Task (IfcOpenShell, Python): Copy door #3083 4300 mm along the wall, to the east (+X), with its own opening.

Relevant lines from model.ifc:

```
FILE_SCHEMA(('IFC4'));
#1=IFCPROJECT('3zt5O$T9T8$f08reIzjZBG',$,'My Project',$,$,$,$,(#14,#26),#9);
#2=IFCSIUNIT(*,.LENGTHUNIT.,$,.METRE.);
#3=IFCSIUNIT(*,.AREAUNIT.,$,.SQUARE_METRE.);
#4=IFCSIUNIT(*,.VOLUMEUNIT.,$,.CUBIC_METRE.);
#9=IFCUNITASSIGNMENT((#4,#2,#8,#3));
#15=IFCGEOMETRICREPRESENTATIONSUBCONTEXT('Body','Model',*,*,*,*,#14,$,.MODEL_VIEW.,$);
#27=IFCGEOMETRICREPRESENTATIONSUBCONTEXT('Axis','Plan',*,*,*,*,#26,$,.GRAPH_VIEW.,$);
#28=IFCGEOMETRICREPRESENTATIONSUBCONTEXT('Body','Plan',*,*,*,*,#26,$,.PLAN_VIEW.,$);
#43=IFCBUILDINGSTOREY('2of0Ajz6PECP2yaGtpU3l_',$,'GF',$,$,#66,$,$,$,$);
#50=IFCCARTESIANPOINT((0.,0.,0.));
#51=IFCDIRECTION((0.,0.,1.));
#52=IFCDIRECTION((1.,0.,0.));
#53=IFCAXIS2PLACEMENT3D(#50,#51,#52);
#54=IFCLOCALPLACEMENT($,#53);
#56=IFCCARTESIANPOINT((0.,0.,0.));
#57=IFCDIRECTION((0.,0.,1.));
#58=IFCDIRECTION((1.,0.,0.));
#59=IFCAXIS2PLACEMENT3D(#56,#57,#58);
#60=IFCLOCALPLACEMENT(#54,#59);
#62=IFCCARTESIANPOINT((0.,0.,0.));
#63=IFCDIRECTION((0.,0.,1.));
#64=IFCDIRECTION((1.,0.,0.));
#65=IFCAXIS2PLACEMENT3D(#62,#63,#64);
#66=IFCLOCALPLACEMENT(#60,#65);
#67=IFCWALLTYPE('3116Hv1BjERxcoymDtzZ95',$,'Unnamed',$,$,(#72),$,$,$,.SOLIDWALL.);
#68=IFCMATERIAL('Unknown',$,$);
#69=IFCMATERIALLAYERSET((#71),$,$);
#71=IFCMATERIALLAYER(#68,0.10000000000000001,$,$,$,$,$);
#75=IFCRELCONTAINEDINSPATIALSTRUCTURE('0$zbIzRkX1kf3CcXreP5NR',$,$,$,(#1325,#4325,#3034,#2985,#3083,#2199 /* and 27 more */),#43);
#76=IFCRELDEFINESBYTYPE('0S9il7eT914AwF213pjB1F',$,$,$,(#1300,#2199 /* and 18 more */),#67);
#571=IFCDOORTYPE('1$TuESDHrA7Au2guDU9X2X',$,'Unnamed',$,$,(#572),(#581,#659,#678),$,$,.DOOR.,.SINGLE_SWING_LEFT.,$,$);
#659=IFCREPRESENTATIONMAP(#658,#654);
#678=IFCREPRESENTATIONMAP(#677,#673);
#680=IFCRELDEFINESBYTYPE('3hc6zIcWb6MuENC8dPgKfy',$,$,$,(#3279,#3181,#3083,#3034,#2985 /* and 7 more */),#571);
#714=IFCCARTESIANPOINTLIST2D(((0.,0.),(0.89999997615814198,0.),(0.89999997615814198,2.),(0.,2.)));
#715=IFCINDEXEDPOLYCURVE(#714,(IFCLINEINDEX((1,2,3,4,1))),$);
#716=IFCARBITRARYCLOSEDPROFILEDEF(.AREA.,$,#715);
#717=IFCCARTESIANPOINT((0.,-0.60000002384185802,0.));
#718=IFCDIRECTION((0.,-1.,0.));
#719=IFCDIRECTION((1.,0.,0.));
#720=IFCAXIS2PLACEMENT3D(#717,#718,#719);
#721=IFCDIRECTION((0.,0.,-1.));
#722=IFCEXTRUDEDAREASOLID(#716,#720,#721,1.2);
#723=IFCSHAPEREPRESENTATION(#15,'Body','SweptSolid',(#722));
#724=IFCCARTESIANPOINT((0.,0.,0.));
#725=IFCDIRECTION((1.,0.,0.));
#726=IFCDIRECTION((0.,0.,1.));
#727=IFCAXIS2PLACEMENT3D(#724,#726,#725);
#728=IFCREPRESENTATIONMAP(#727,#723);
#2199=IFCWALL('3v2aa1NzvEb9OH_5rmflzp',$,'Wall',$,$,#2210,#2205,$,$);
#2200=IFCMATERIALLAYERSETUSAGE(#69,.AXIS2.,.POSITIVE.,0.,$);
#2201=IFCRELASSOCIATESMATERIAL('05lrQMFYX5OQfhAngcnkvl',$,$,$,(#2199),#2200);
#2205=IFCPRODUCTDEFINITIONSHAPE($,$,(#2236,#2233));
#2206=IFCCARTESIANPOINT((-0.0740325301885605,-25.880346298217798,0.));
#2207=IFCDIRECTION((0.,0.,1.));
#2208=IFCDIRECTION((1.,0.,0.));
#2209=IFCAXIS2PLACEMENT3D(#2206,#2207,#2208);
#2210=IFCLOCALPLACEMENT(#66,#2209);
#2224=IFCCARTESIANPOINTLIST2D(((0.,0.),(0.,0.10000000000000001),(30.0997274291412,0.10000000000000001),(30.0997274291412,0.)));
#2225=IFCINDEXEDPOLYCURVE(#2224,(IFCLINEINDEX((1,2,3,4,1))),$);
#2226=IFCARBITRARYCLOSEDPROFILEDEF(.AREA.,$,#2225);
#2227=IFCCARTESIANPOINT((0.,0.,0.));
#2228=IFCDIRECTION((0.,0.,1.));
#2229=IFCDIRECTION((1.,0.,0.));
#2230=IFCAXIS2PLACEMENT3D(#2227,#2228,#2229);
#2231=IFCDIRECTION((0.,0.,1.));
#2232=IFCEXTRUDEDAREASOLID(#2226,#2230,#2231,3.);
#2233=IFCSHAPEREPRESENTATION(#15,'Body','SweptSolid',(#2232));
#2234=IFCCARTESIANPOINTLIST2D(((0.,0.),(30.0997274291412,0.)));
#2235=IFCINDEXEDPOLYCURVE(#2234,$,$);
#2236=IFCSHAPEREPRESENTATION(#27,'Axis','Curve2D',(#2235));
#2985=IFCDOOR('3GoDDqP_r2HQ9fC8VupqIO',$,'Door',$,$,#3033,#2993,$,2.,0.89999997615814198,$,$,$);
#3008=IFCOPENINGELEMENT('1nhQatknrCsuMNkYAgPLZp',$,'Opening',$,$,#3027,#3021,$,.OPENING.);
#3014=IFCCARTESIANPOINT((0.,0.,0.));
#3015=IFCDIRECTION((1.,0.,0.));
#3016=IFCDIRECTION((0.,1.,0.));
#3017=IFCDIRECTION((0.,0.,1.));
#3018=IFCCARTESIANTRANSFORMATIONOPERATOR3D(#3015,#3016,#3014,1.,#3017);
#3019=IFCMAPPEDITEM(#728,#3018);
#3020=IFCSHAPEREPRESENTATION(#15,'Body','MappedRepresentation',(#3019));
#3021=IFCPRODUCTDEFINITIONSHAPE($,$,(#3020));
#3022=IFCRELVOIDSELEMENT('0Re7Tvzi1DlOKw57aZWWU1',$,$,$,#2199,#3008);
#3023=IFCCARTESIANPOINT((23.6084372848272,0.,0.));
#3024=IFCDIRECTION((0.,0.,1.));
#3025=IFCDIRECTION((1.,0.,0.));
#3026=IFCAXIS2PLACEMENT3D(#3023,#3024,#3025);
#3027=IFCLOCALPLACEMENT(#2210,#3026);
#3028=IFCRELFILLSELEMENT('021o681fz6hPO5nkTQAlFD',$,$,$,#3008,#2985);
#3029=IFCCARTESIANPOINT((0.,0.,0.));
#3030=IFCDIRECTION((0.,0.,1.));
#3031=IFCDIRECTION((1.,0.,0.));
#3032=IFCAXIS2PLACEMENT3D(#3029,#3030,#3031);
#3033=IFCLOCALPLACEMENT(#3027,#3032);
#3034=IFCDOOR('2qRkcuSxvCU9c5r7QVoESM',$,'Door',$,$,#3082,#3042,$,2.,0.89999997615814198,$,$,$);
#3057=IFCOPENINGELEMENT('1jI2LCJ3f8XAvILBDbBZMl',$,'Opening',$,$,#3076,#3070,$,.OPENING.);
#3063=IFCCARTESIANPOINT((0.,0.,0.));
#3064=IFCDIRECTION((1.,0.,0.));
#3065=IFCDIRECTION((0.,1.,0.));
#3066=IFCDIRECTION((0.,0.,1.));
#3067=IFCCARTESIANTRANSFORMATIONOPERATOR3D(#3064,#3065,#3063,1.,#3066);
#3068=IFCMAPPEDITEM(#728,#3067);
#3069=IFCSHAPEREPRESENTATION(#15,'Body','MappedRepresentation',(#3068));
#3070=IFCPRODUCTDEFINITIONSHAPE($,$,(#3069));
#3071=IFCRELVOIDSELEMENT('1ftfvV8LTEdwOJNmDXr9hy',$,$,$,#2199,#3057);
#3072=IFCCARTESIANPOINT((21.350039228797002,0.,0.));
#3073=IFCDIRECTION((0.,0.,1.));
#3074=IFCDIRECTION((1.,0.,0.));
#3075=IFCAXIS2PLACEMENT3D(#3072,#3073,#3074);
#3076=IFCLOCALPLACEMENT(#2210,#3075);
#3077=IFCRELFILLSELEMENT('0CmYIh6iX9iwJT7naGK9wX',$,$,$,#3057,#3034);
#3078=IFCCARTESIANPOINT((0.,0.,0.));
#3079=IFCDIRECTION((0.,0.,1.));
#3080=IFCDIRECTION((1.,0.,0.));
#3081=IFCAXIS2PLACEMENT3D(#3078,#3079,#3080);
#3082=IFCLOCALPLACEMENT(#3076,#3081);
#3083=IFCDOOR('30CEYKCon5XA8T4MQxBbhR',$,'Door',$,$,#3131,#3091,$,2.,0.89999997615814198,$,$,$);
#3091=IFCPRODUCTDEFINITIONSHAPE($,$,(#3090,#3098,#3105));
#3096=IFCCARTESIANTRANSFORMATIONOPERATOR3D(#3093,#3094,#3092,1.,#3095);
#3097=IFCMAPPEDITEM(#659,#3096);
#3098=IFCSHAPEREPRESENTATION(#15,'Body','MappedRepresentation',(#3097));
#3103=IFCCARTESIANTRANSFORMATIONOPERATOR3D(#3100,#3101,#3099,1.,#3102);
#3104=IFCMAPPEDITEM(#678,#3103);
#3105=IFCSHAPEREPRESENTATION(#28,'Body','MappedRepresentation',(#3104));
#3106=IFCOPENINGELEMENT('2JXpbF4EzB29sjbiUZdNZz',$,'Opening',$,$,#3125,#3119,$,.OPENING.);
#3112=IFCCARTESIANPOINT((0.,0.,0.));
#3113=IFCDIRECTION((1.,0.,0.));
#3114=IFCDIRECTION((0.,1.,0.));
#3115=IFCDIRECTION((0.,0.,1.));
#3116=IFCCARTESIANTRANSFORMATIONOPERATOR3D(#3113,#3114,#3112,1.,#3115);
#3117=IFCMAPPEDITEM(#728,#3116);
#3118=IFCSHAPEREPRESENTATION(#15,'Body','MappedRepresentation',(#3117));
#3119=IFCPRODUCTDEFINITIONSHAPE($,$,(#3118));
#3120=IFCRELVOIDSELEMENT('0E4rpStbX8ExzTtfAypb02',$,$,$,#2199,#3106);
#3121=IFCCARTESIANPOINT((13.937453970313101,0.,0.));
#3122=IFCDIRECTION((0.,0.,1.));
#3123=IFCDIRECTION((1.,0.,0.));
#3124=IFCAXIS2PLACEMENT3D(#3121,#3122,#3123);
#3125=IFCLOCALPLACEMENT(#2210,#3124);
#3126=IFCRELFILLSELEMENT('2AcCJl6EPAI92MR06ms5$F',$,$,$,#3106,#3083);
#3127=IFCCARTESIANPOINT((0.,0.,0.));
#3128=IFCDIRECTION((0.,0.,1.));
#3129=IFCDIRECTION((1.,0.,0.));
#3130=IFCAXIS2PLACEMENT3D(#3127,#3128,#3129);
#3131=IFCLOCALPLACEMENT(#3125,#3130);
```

```python
import ifcopenshell
import ifcopenshell.api.feature
import ifcopenshell.api.geometry
import ifcopenshell.api.root
import ifcopenshell.geom
import ifcopenshell.util.element
import ifcopenshell.util.placement
import ifcopenshell.util.shape
import ifcopenshell.util.unit

model = ifcopenshell.open("model.ifc")
unit_scale = ifcopenshell.util.unit.calculate_unit_scale(model)
settings = ifcopenshell.geom.settings()


def volume(element):
    """Net volume in cubic metres, openings subtracted."""
    shape = ifcopenshell.geom.create_shape(settings, element)
    return ifcopenshell.util.shape.get_volume(shape.geometry)


door = model.by_guid("30CEYKCon5XA8T4MQxBbhR")
opening = door.FillsVoids[0].RelatingOpeningElement
wall = opening.VoidsElements[0].RelatingBuildingElement
before = volume(wall)
shift = ifcopenshell.util.placement.get_local_placement(wall.ObjectPlacement)[:3, 0] * 4.3 / unit_scale

# copy_class copies the void relationship, type, container and properties, but no geometry.
new_opening = ifcopenshell.api.root.copy_class(model, product=opening)
new_opening.Representation = ifcopenshell.util.element.copy_deep(
    model, opening.Representation, exclude=["IfcGeometricRepresentationContext", "IfcRepresentationMap"]
)
new_door = ifcopenshell.api.root.copy_class(model, product=door)
new_door.Representation = ifcopenshell.util.element.copy_deep(
    model, door.Representation, exclude=["IfcGeometricRepresentationContext", "IfcRepresentationMap"]
)
ifcopenshell.api.feature.add_filling(model, opening=new_opening, element=new_door)

for old, new in ((opening, new_opening), (door, new_door)):
    matrix = ifcopenshell.util.placement.get_local_placement(old.ObjectPlacement)
    matrix[:3, 3] += shift
    ifcopenshell.api.geometry.edit_object_placement(model, product=new, matrix=matrix, is_si=False)

after = volume(wall)

print(f"wall volume {before:.3f} -> {after:.3f} m3")

model.write("model_updated.ifc")
```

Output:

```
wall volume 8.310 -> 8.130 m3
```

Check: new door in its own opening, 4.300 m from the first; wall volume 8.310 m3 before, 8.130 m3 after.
